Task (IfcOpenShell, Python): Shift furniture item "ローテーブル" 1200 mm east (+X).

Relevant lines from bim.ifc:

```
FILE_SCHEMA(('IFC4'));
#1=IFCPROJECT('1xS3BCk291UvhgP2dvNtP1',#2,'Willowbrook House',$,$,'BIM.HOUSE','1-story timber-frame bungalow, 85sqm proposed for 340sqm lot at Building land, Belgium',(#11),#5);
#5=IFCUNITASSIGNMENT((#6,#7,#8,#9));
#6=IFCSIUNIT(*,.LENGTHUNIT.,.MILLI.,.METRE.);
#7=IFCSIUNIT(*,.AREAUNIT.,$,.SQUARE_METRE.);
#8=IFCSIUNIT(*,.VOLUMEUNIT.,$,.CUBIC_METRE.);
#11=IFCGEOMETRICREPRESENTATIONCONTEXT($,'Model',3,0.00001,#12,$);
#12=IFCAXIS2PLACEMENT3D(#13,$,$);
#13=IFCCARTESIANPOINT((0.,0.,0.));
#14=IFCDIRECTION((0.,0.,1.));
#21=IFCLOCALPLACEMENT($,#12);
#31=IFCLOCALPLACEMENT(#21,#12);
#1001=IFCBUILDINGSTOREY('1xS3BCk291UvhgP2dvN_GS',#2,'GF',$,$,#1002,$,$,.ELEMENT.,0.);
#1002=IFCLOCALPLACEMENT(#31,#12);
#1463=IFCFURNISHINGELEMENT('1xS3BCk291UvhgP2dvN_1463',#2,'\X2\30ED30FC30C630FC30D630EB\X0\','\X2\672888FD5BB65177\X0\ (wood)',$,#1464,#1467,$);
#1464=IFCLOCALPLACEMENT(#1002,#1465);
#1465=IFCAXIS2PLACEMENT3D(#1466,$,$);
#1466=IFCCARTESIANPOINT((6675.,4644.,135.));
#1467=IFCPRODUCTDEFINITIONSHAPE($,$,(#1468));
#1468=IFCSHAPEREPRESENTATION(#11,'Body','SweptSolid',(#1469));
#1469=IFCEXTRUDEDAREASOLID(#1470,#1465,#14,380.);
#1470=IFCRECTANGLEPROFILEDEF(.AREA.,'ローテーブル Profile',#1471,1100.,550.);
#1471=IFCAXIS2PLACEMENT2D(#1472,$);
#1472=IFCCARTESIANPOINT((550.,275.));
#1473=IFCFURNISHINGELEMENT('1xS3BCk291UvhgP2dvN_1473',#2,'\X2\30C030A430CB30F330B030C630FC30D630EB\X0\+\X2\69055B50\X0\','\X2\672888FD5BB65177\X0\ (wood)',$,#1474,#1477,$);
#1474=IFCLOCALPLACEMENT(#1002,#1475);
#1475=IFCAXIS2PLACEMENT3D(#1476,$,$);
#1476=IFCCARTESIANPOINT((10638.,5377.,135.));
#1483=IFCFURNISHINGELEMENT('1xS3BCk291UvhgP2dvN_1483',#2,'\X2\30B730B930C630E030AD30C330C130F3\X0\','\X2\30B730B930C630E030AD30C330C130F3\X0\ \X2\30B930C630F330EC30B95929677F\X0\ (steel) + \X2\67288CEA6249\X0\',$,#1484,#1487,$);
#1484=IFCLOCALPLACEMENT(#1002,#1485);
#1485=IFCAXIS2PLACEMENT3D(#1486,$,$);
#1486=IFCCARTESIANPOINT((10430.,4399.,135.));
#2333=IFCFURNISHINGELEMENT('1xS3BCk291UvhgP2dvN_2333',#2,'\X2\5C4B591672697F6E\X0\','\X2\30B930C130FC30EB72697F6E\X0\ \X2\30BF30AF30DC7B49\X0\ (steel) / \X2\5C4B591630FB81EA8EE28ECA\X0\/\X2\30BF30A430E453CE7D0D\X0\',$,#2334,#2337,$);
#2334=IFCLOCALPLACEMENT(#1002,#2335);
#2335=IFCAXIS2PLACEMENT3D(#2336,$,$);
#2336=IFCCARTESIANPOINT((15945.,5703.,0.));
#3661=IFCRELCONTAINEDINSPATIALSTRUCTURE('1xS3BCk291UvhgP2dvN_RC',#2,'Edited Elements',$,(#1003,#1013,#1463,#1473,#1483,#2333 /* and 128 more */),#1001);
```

```python
import ifcopenshell
import ifcopenshell.api.geometry
import ifcopenshell.util.placement
import ifcopenshell.util.unit

model = ifcopenshell.open("bim.ifc")
unit_scale = ifcopenshell.util.unit.calculate_unit_scale(model)

item = model.by_id(1463)
matrix = ifcopenshell.util.placement.get_local_placement(item.ObjectPlacement)
matrix[0, 3] += 1.2 / unit_scale
ifcopenshell.api.geometry.edit_object_placement(model, product=item, matrix=matrix, is_si=False)

print(ifcopenshell.util.placement.get_local_placement(item.ObjectPlacement).round(3) + 0.0)

model.write("bim_rev.ifc")
```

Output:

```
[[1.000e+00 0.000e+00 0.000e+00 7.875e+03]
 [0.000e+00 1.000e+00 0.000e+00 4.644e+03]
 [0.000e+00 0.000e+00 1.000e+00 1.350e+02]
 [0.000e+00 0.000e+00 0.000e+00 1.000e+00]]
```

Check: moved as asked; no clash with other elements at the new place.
